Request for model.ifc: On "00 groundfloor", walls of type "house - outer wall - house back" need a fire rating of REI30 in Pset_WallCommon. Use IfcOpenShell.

First a look at what the model holds.

```python
import ifcopenshell
import ifcopenshell.util.element

model = ifcopenshell.open("model.ifc")
print(model.schema)
storey = next(s for s in model.by_type("IfcBuildingStorey") if s.Name == "00 groundfloor")
walls = [e for e in ifcopenshell.util.element.get_decomposition(storey) if e.is_a("IfcWall")]
seen = {}
for e in walls:
    element_type = ifcopenshell.util.element.get_type(e)
    key = (element_type.Name if element_type != e and element_type else None, ifcopenshell.util.element.get_pset(e, "Pset_WallCommon", "FireRating"))
    seen[key] = seen.get(key, 0) + 1
for (name, value), count in sorted(seen.items(), key=str):
    print(count, "x", name, "|", value)
```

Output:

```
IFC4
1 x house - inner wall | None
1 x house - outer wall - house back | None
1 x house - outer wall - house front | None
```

```python
import ifcopenshell
import ifcopenshell.api.pset
import ifcopenshell.util.element

model = ifcopenshell.open("model.ifc")

storey = next(s for s in model.by_type("IfcBuildingStorey") if s.Name == "00 groundfloor")
walls = [e for e in ifcopenshell.util.element.get_decomposition(storey) if e.is_a("IfcWall")]

count = 0
for e in walls:
    element_type = ifcopenshell.util.element.get_type(e)
    if element_type in (None, e) or element_type.Name != "house - outer wall - house back":
        continue
    # add_pset returns the element's existing set when there is one.
    pset = ifcopenshell.api.pset.add_pset(model, product=e, name="Pset_WallCommon")
    ifcopenshell.api.pset.edit_pset(model, pset=pset, properties={"FireRating": "REI30"})
    count += 1

print(count, "walls updated")

model.write("model_updated.ifc")
```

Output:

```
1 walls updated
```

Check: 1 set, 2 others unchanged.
